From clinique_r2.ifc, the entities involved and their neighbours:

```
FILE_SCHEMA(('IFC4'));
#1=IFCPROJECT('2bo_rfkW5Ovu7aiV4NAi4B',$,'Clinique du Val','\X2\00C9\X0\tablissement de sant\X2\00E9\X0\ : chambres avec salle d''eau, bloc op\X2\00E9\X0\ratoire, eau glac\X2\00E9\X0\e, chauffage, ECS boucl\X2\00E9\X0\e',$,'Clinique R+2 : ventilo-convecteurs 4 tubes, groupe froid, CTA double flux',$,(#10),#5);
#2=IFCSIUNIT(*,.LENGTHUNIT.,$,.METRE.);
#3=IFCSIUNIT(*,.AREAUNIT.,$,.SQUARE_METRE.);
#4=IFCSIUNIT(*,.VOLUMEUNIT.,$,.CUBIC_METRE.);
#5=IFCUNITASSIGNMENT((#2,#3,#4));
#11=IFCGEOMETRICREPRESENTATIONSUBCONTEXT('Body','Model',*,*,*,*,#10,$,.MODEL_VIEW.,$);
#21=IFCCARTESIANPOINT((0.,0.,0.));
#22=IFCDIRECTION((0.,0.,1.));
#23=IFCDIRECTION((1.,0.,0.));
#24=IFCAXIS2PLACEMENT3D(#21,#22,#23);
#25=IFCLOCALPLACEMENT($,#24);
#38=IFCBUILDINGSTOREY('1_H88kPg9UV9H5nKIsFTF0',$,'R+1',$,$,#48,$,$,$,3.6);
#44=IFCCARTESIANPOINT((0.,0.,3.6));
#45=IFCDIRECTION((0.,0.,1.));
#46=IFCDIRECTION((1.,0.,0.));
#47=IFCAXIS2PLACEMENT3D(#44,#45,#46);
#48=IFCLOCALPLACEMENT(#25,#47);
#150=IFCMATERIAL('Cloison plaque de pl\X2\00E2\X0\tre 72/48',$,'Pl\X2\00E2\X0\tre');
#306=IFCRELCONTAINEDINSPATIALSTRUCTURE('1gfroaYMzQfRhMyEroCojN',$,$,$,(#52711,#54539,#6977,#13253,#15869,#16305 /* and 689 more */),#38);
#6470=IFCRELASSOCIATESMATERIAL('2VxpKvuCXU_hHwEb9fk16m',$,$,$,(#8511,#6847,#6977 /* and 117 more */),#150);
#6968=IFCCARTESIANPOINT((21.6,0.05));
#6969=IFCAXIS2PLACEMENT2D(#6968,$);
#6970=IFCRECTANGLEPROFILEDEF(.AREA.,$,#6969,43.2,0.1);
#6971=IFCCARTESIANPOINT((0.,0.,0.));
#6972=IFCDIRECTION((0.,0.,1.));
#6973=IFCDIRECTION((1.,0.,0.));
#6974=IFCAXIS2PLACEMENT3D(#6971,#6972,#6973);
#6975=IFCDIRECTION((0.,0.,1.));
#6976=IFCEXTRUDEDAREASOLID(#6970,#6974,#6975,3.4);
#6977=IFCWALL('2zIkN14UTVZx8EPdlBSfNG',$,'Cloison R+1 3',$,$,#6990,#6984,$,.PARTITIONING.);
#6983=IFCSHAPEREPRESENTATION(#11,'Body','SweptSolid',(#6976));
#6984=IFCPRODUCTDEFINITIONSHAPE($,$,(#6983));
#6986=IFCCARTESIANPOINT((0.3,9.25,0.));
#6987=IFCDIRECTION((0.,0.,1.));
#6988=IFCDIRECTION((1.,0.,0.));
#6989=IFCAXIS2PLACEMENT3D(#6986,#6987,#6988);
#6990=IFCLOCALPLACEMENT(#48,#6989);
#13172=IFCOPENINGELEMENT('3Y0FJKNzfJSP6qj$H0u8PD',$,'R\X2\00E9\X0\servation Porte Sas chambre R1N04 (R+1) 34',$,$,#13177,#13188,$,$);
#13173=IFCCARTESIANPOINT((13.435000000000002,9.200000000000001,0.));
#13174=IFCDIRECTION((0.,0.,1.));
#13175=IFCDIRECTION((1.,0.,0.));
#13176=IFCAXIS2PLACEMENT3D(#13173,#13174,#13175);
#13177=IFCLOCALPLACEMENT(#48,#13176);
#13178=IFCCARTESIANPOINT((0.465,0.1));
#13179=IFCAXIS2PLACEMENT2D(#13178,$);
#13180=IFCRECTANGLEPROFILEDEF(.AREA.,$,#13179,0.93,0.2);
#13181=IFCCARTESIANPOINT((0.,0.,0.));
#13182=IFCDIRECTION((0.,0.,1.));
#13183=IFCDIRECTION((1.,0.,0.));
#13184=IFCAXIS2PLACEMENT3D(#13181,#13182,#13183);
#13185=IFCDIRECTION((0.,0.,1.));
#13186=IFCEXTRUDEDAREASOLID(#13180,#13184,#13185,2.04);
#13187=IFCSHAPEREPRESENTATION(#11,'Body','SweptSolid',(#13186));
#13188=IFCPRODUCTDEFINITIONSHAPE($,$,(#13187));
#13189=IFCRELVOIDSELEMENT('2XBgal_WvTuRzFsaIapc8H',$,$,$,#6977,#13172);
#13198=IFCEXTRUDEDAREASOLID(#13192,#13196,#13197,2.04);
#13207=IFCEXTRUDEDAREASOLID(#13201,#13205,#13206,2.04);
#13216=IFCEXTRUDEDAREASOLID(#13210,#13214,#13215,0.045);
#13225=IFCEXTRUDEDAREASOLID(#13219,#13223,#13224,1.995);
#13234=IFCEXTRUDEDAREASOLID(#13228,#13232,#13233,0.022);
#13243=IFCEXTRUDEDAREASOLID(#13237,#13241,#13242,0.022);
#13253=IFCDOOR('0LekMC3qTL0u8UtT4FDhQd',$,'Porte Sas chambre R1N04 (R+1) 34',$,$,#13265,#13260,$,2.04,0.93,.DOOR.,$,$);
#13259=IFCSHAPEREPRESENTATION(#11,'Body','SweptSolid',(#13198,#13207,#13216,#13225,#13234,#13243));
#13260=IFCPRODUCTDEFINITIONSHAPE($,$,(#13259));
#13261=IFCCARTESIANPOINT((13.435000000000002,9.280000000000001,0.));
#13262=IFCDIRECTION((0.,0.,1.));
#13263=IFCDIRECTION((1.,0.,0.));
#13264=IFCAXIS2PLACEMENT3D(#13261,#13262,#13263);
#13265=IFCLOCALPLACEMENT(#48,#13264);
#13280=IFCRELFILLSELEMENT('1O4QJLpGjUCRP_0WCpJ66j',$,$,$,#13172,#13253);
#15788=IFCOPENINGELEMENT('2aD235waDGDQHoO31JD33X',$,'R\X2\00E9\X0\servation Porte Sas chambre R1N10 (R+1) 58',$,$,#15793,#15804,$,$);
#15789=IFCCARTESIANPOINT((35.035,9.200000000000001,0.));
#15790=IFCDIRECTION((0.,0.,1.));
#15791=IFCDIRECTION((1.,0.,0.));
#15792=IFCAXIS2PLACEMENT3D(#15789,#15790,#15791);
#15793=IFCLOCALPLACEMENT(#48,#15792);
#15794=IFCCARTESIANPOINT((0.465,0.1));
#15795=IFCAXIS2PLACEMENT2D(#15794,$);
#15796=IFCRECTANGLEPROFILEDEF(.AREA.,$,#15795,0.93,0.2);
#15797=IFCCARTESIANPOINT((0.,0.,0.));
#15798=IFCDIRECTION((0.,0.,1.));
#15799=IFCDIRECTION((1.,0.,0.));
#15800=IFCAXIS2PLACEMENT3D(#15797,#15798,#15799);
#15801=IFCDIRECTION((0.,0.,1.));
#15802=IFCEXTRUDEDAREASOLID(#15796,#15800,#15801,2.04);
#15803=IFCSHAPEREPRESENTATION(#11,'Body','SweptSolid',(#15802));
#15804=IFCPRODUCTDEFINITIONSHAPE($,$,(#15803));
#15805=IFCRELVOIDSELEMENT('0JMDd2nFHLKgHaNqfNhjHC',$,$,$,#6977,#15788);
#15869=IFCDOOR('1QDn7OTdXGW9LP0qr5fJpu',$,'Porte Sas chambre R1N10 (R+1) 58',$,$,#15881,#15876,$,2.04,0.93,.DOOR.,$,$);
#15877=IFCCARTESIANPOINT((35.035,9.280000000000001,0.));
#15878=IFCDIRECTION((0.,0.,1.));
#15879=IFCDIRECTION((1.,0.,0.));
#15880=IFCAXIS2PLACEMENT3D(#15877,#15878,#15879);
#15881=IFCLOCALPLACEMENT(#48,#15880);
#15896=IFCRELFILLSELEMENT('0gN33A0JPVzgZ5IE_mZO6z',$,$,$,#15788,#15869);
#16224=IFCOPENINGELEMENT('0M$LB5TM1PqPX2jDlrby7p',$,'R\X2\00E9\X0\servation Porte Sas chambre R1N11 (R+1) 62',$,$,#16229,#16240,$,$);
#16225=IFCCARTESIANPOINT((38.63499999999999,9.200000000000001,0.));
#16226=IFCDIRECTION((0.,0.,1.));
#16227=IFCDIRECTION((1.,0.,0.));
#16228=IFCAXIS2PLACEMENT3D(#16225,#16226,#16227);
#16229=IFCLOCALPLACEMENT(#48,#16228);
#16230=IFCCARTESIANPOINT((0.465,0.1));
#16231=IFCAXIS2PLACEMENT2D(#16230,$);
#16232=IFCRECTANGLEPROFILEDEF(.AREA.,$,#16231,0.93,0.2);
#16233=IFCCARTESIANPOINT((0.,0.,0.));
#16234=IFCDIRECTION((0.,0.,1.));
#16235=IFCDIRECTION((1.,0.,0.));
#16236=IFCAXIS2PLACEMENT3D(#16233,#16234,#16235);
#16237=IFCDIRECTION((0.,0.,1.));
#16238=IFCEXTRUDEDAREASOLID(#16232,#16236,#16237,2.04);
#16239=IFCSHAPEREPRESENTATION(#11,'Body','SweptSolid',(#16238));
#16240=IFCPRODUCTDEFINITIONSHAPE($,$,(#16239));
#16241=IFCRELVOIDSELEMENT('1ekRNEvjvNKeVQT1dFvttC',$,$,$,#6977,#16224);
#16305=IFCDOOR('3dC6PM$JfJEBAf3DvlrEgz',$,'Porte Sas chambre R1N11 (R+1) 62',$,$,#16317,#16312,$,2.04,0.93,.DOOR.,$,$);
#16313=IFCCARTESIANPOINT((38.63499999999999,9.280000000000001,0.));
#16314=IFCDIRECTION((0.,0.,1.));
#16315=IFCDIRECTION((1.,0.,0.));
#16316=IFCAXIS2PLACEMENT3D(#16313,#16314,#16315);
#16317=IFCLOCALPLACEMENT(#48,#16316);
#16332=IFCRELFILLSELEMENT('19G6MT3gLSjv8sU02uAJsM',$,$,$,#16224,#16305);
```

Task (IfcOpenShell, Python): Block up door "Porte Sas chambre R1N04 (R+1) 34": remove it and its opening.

```python
import ifcopenshell
import ifcopenshell.api.feature
import ifcopenshell.api.root
import ifcopenshell.geom
import ifcopenshell.util.shape

model = ifcopenshell.open("clinique_r2.ifc")
settings = ifcopenshell.geom.settings()


def volume(element):
    """Net volume in cubic metres, openings subtracted."""
    shape = ifcopenshell.geom.create_shape(settings, element)
    return ifcopenshell.util.shape.get_volume(shape.geometry)


door = model.by_guid("0LekMC3qTL0u8UtT4FDhQd")
opening = door.FillsVoids[0].RelatingOpeningElement
wall = opening.VoidsElements[0].RelatingBuildingElement
before = volume(wall)

ifcopenshell.api.root.remove_product(model, product=door)
ifcopenshell.api.feature.remove_feature(model, feature=opening)

after = volume(wall)

print(f"wall volume {before:.3f} -> {after:.3f} m3")

model.write("clinique_r2-out.ifc")
```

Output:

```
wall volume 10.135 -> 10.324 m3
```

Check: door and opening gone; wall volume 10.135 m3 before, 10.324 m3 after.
